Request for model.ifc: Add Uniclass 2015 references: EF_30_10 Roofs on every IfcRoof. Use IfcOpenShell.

First a look at what the model holds.

```python
import ifcopenshell

model = ifcopenshell.open("model.ifc")
print(model.schema)
print("classifications:", [c.Name for c in model.by_type("IfcClassification")])
for ifc_class in ("IfcDoor", "IfcRoof", "IfcStair", "IfcWall", "IfcWindow"):
    print(ifc_class, len(model.by_type(ifc_class)))
```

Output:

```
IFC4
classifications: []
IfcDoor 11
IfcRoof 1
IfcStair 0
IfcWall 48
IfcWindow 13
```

```python
import ifcopenshell
import ifcopenshell.api.classification

model = ifcopenshell.open("model.ifc")

system = ifcopenshell.api.classification.add_classification(model, classification="Uniclass 2015")

codes = {
    "IfcRoof": ("EF_30_10", "Roofs"),
}
for ifc_class, (code, name) in codes.items():
    products = model.by_type(ifc_class)
    ifcopenshell.api.classification.add_reference(
        model, products=products, classification=system, identification=code, name=name
    )
    print(code, len(products))

model.write("model_v2.ifc")
```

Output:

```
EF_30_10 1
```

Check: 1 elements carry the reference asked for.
